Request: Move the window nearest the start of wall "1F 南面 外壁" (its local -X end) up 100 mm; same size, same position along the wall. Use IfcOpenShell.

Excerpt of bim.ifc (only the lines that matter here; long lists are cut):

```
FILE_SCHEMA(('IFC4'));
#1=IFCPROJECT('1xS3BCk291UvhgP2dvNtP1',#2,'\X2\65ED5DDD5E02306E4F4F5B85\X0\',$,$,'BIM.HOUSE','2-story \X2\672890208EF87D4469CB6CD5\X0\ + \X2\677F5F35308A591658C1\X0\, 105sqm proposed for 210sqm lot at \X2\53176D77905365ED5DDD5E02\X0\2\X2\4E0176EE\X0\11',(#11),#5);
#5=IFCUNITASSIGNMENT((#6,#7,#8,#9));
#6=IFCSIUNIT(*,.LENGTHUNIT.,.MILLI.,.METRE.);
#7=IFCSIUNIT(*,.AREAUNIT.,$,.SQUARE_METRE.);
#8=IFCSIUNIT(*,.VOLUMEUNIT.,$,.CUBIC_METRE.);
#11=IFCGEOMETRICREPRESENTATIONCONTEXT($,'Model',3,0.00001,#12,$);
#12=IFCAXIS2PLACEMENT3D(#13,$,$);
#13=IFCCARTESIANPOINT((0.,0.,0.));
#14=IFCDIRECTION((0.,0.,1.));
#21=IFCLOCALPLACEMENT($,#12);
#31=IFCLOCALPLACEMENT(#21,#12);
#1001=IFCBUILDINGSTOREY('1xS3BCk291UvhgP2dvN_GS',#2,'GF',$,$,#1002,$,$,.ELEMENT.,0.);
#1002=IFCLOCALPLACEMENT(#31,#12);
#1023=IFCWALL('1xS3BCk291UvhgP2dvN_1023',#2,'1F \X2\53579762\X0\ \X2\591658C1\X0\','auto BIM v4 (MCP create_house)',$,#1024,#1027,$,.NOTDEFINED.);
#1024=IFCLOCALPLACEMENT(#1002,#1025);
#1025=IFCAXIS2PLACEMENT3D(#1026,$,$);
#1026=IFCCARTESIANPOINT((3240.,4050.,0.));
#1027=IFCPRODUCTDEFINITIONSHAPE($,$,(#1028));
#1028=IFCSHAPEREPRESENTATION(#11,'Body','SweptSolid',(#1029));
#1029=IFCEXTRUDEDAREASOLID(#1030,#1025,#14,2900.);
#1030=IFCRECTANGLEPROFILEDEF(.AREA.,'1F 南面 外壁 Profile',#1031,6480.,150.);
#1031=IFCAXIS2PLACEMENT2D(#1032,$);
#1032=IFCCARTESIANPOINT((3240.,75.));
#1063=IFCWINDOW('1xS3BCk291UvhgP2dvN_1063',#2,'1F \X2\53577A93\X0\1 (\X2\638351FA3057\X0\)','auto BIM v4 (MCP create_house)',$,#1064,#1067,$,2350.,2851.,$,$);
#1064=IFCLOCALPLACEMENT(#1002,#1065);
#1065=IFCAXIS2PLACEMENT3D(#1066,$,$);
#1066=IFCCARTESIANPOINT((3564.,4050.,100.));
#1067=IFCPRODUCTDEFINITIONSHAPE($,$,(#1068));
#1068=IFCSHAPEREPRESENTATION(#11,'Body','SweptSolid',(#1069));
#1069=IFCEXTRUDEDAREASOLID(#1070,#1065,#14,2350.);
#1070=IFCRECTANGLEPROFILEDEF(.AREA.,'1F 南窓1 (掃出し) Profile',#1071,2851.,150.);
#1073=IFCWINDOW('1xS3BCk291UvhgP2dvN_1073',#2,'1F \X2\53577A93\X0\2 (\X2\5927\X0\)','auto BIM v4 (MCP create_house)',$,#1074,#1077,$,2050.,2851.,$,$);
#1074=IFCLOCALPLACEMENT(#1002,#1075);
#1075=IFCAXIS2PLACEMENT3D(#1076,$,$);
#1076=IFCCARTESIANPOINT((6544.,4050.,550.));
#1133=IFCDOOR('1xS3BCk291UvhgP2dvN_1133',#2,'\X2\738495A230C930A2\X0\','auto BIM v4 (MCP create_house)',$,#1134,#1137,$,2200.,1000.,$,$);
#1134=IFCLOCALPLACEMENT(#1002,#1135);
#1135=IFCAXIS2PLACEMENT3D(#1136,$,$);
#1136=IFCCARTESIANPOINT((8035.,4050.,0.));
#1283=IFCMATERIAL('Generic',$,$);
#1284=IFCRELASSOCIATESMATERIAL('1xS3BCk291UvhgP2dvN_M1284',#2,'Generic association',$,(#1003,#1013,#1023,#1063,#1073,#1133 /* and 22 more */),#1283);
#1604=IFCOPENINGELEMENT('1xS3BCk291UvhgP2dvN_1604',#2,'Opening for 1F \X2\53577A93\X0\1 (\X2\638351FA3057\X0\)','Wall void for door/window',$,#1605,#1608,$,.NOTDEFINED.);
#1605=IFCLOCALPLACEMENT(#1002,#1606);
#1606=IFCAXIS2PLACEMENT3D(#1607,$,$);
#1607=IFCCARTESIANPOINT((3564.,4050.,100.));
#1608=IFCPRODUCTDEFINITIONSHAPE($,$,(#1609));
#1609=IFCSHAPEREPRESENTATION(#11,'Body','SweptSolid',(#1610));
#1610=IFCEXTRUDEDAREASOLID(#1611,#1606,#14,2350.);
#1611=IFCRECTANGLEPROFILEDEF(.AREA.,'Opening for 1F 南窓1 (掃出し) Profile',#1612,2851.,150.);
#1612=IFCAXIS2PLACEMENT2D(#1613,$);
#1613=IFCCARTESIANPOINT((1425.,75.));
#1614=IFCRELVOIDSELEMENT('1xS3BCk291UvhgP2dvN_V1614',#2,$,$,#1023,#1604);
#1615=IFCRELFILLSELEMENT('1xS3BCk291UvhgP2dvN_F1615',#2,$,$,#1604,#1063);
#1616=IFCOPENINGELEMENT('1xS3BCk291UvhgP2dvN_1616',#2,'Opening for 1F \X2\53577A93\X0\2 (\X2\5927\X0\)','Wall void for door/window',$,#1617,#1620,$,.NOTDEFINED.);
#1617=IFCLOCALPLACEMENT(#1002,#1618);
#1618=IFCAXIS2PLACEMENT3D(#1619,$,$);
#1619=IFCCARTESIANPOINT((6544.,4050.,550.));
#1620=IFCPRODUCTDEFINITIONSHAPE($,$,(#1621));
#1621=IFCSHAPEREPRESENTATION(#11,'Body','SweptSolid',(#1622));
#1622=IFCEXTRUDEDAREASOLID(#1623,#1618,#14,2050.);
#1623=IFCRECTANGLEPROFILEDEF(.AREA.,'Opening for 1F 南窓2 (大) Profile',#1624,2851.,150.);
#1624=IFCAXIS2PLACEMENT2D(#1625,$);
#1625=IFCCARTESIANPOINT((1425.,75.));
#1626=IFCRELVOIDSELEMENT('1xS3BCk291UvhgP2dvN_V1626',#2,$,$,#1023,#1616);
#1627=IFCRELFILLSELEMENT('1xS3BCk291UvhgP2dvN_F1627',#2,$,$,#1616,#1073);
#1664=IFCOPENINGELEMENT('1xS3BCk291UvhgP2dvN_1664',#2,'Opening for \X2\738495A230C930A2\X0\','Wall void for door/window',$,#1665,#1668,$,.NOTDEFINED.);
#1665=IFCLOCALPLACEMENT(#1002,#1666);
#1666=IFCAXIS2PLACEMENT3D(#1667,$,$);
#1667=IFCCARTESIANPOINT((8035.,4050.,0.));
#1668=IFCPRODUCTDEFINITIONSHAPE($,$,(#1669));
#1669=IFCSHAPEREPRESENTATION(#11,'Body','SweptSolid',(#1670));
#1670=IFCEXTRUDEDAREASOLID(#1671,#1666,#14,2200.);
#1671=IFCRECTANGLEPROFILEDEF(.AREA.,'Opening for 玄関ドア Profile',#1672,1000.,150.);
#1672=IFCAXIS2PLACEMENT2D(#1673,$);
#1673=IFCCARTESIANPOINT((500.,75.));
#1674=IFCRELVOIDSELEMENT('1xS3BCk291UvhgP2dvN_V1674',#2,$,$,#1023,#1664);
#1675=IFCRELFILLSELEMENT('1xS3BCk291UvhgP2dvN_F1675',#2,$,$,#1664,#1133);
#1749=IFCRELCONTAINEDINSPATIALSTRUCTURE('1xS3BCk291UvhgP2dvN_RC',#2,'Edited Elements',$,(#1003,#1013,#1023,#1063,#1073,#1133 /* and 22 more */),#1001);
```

```python
import numpy as np
import ifcopenshell
import ifcopenshell.api.geometry
import ifcopenshell.util.placement
import ifcopenshell.util.unit

model = ifcopenshell.open("bim.ifc")
unit_scale = ifcopenshell.util.unit.calculate_unit_scale(model)

window = model.by_id(1063)
opening = window.FillsVoids[0].RelatingOpeningElement
dz = 100.0

shift = np.array([0.0, 0.0, dz])
# The window is not placed relative to its opening, so move both.
for product in (opening, window):
    matrix = ifcopenshell.util.placement.get_local_placement(product.ObjectPlacement)
    matrix[:3, 3] += shift
    ifcopenshell.api.geometry.edit_object_placement(model, product=product, matrix=matrix, is_si=False)

print(f"moved by {dz * unit_scale:+.3f} m")

model.write("bim_edited.ifc")
```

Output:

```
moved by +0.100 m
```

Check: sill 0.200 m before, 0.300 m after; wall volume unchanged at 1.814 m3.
